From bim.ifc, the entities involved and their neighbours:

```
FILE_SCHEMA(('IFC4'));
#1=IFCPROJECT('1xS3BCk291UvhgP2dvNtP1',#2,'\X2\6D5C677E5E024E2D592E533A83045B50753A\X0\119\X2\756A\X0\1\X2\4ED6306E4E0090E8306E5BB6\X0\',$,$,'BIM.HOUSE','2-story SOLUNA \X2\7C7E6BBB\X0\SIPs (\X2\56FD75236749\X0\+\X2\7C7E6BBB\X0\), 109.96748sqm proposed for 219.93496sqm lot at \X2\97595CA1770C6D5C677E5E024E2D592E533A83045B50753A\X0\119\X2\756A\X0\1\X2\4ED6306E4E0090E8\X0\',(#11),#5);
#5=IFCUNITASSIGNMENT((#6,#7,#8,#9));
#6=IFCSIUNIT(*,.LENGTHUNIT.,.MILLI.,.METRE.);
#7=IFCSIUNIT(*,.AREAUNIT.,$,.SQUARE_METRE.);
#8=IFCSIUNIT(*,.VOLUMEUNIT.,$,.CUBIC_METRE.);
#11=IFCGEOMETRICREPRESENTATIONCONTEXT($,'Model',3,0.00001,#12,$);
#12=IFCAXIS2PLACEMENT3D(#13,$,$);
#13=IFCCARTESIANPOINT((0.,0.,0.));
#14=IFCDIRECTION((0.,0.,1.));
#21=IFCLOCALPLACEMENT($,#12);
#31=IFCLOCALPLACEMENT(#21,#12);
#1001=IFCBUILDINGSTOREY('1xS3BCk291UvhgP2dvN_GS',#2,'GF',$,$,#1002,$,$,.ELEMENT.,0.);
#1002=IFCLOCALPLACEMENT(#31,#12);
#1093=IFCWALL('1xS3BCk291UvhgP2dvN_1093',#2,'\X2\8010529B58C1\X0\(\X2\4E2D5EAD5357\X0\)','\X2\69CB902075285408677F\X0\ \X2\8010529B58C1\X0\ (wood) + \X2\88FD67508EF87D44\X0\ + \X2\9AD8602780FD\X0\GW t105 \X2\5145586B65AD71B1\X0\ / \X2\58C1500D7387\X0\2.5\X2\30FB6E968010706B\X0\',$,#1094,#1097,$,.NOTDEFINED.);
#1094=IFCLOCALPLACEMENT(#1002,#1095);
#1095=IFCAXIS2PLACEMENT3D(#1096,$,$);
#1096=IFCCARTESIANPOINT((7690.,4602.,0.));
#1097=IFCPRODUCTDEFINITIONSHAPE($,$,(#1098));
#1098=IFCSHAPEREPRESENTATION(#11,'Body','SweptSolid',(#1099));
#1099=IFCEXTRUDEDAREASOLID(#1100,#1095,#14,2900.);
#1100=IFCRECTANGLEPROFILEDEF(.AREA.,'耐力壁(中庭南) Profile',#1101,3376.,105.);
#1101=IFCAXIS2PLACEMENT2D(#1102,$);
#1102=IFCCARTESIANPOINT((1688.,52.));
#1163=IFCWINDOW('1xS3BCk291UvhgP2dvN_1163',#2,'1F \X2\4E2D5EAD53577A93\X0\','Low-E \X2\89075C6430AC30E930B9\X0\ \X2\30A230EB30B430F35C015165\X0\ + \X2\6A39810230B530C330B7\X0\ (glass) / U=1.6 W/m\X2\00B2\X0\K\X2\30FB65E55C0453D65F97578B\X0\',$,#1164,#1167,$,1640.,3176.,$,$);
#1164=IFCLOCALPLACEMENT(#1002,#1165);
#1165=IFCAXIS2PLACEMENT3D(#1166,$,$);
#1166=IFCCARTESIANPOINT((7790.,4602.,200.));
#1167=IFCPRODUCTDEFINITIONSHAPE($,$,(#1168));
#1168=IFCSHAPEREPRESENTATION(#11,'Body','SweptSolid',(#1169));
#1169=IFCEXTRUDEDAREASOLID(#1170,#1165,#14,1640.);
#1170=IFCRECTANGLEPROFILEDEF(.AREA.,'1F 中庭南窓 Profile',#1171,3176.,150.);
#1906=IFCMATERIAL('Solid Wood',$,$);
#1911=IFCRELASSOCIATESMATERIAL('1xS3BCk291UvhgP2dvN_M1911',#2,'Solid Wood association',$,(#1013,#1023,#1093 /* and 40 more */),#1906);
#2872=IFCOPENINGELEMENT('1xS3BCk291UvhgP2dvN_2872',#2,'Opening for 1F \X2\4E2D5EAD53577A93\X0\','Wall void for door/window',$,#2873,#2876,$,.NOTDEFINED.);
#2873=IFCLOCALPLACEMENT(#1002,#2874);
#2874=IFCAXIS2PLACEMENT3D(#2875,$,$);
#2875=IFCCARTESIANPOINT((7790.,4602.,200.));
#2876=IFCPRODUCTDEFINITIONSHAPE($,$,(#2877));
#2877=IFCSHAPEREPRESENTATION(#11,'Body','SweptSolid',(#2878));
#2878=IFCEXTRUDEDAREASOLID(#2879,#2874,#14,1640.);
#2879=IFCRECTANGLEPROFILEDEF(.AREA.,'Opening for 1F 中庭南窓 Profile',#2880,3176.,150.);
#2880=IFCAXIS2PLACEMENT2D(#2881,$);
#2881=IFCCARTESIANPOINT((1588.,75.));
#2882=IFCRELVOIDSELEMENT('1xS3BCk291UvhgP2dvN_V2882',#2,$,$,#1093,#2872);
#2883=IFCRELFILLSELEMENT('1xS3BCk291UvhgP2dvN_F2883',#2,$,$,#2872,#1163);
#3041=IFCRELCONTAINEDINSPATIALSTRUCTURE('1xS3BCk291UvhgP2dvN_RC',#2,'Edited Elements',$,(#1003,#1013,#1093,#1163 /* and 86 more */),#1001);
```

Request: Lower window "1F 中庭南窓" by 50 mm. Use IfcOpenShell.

```python
import numpy as np
import ifcopenshell
import ifcopenshell.api.geometry
import ifcopenshell.util.placement
import ifcopenshell.util.unit

model = ifcopenshell.open("bim.ifc")
unit_scale = ifcopenshell.util.unit.calculate_unit_scale(model)

window = model.by_guid("1xS3BCk291UvhgP2dvN_1163")
opening = window.FillsVoids[0].RelatingOpeningElement
dz = -0.05 / unit_scale

shift = np.array([0.0, 0.0, dz])
# The window is not placed relative to its opening, so move both.
for product in (opening, window):
    matrix = ifcopenshell.util.placement.get_local_placement(product.ObjectPlacement)
    matrix[:3, 3] += shift
    ifcopenshell.api.geometry.edit_object_placement(model, product=product, matrix=matrix, is_si=False)

print(f"moved by {dz * unit_scale:+.3f} m")

model.write("bim-out.ifc")
```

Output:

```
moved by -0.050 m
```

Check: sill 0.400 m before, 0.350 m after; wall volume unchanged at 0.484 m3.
